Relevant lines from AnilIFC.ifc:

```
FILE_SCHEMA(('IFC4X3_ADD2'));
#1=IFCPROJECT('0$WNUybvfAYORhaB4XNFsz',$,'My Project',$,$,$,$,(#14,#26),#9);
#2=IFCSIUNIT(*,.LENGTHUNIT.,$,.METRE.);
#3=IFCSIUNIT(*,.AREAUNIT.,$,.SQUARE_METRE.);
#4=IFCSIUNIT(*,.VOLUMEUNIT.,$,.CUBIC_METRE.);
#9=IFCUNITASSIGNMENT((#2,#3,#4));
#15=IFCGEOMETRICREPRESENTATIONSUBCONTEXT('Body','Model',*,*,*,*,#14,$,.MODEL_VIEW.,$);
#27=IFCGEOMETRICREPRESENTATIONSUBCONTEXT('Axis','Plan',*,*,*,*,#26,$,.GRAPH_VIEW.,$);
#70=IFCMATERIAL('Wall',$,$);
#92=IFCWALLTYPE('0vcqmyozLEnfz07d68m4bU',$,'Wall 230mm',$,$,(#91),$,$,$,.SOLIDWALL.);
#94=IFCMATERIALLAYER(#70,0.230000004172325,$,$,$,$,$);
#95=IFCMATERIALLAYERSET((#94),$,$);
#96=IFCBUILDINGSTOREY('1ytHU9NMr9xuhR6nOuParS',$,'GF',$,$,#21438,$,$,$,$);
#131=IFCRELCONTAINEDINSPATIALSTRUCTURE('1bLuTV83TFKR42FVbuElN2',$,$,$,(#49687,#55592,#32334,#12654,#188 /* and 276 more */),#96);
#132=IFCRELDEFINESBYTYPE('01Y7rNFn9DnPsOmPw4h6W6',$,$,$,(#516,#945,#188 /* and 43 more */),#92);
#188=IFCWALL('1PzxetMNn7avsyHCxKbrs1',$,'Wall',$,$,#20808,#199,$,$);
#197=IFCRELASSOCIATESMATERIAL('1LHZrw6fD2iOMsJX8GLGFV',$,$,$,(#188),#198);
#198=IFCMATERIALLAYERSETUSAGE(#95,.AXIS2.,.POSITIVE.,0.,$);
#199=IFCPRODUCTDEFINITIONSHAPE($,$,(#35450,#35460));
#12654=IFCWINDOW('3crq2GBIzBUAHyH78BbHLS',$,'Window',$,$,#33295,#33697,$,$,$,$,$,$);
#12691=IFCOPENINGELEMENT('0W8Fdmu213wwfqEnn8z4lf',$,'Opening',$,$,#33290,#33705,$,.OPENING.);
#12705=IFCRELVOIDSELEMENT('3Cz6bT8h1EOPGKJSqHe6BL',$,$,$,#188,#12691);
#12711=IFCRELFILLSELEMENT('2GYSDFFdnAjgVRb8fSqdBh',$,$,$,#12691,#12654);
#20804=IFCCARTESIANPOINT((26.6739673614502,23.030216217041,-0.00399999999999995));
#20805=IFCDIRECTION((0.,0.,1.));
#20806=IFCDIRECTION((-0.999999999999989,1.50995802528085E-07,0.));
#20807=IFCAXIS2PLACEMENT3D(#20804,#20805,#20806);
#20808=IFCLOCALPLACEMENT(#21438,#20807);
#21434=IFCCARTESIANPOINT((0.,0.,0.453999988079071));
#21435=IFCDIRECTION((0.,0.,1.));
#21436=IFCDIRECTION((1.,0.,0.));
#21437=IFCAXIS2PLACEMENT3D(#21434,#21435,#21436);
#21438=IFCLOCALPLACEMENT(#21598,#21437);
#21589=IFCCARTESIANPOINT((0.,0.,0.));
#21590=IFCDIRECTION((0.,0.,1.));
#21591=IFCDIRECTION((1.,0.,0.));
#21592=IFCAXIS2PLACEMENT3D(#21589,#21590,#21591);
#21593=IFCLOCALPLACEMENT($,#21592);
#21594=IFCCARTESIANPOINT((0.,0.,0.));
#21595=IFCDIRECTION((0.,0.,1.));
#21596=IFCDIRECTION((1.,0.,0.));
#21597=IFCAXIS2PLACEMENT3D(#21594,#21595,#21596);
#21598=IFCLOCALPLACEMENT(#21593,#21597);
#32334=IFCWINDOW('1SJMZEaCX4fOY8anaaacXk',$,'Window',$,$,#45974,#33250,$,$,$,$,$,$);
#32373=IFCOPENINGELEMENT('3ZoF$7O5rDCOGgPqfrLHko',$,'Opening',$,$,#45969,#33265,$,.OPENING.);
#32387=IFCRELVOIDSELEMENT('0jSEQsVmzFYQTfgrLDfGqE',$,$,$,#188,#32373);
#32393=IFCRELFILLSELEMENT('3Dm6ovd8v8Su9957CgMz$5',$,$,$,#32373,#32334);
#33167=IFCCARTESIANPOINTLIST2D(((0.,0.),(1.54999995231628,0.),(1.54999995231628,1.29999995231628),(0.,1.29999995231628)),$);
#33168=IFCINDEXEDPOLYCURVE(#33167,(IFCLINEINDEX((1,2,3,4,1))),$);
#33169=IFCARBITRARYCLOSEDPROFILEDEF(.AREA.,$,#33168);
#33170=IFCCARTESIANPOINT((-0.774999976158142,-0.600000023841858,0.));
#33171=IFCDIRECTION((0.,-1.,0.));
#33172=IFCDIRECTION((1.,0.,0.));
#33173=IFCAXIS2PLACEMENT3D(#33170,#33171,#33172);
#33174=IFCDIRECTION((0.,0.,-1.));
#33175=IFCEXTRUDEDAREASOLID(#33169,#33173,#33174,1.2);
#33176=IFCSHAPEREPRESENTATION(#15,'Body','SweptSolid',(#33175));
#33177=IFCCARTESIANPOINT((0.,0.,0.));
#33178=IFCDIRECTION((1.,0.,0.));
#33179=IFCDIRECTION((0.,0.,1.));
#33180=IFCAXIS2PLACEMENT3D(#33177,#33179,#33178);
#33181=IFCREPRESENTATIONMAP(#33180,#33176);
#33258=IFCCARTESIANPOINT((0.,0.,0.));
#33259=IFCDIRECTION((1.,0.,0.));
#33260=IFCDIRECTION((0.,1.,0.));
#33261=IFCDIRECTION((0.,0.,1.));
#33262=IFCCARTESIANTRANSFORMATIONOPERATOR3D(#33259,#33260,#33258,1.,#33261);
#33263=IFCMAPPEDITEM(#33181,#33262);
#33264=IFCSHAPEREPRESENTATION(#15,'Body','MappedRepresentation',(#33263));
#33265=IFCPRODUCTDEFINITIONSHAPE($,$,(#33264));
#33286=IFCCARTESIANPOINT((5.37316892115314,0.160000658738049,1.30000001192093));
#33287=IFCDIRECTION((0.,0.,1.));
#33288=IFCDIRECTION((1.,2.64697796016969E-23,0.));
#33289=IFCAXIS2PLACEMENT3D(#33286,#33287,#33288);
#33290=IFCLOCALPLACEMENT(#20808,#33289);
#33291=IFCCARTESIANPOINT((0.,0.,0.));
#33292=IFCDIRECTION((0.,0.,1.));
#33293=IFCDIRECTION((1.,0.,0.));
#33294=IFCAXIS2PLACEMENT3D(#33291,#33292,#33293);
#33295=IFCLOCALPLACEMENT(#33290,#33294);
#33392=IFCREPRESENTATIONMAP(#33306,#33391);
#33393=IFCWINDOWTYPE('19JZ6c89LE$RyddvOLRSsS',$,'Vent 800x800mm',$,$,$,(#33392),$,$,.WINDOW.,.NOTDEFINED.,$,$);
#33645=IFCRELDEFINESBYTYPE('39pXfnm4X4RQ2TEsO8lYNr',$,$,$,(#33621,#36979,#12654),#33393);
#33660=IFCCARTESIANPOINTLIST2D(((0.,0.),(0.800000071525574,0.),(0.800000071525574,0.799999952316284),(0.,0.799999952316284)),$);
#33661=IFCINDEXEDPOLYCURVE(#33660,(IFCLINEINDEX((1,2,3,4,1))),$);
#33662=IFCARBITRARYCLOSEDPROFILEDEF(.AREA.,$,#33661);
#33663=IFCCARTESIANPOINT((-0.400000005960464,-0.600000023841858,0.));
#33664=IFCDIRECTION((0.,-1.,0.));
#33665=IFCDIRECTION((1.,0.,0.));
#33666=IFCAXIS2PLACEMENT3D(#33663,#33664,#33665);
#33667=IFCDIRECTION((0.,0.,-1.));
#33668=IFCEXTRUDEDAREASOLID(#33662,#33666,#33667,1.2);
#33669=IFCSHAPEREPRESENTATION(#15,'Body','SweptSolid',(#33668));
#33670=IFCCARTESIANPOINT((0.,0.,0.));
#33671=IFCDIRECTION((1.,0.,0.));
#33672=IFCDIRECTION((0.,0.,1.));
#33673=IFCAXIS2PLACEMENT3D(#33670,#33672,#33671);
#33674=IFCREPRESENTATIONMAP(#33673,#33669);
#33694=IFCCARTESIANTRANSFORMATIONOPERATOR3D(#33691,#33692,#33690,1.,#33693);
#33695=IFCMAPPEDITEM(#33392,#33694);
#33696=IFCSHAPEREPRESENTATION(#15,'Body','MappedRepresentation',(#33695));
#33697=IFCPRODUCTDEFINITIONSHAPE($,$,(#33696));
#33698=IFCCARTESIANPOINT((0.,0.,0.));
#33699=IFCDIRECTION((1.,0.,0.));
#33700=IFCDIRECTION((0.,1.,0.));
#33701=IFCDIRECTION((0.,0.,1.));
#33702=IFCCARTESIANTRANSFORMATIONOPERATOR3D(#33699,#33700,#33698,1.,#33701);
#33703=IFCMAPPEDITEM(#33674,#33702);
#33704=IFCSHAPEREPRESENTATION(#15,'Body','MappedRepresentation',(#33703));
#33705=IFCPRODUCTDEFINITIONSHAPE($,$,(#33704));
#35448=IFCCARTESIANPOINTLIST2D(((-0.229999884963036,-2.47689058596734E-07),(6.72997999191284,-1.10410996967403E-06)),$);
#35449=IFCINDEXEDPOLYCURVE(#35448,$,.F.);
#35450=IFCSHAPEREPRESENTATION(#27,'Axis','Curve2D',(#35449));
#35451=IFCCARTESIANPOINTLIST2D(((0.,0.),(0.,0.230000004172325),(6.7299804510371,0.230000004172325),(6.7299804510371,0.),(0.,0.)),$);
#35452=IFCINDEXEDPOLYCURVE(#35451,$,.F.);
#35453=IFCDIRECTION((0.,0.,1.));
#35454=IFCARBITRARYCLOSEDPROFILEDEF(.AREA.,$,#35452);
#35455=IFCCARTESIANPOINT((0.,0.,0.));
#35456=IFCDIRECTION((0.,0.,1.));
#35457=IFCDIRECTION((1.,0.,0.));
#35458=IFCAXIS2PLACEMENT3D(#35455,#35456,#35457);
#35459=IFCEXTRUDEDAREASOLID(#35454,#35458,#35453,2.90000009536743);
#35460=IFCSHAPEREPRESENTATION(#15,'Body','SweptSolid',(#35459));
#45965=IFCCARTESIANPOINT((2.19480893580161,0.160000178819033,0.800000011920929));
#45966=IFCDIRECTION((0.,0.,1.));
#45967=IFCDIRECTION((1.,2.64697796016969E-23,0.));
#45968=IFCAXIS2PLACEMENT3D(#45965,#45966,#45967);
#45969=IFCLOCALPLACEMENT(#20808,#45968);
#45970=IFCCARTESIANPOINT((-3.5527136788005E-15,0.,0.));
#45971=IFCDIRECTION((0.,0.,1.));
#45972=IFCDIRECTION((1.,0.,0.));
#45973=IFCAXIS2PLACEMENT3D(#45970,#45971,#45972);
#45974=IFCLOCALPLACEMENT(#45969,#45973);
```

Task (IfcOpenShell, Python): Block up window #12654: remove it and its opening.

```python
import ifcopenshell
import ifcopenshell.api.feature
import ifcopenshell.api.root
import ifcopenshell.geom
import ifcopenshell.util.shape

model = ifcopenshell.open("AnilIFC.ifc")
settings = ifcopenshell.geom.settings()


def volume(element):
    """Net volume in cubic metres, openings subtracted."""
    shape = ifcopenshell.geom.create_shape(settings, element)
    return ifcopenshell.util.shape.get_volume(shape.geometry)


window = model.by_guid("3crq2GBIzBUAHyH78BbHLS")
opening = window.FillsVoids[0].RelatingOpeningElement
wall = opening.VoidsElements[0].RelatingBuildingElement
before = volume(wall)

ifcopenshell.api.root.remove_product(model, product=window)
ifcopenshell.api.feature.remove_feature(model, feature=opening)

after = volume(wall)

print(f"wall volume {before:.3f} -> {after:.3f} m3")

model.write("AnilIFC-out.ifc")
```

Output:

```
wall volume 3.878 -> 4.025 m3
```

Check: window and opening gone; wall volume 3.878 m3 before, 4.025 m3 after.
